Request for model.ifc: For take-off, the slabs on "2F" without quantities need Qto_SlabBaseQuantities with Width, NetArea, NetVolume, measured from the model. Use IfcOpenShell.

First a look at what the model holds.

```python
import ifcopenshell
import ifcopenshell.util.element
import ifcopenshell.util.unit

model = ifcopenshell.open("model.ifc")
print(model.schema)
for unit_type in ("LENGTHUNIT", "AREAUNIT", "VOLUMEUNIT"):
    print(unit_type, ifcopenshell.util.unit.calculate_unit_scale(model, unit_type))
storey = next(s for s in model.by_type("IfcBuildingStorey") if s.Name == "2F")
slabs = [e for e in ifcopenshell.util.element.get_decomposition(storey) if e.is_a("IfcSlab")]
for e in sorted(slabs, key=lambda e: e.id()):
    print(e.id(), e.is_a(), e.Name, list(ifcopenshell.util.element.get_psets(e, qtos_only=True)), sep=" | ")
```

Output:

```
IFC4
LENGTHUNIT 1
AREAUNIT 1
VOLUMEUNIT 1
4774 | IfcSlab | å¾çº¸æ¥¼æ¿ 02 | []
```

```python
import ifcopenshell
import ifcopenshell.api.pset
import ifcopenshell.geom
import ifcopenshell.util.element
import ifcopenshell.util.shape
import ifcopenshell.util.unit

model = ifcopenshell.open("model.ifc")
unit_scale = ifcopenshell.util.unit.calculate_unit_scale(model)
area_scale = ifcopenshell.util.unit.calculate_unit_scale(model, "AREAUNIT")
volume_scale = ifcopenshell.util.unit.calculate_unit_scale(model, "VOLUMEUNIT")
settings = ifcopenshell.geom.settings()

storey = next(s for s in model.by_type("IfcBuildingStorey") if s.Name == "2F")
slabs = [e for e in ifcopenshell.util.element.get_decomposition(storey) if e.is_a("IfcSlab")]

for e in sorted(slabs, key=lambda e: e.id()):
    if ifcopenshell.util.element.get_psets(e, qtos_only=True, should_inherit=False):
        continue
    # Geometry comes back in metres, in the element's own axes.
    shape = ifcopenshell.geom.create_shape(settings, e)
    values = {
        "Width": ifcopenshell.util.shape.get_z(shape.geometry) / unit_scale,
        "NetArea": ifcopenshell.util.shape.get_footprint_area(shape.geometry) / area_scale,
        "NetVolume": ifcopenshell.util.shape.get_volume(shape.geometry) / volume_scale,
    }
    qto = ifcopenshell.api.pset.add_qto(model, product=e, name="Qto_SlabBaseQuantities")
    ifcopenshell.api.pset.edit_qto(model, qto=qto, properties=values)
    print(e.id(), {k: round(v, 3) for k, v in values.items()})

model.write("model_updated.ifc")
```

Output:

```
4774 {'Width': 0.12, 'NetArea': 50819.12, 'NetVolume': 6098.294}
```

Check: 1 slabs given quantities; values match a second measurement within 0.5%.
